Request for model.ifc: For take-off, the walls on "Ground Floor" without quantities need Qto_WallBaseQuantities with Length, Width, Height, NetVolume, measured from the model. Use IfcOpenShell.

First a look at what the model holds.

```python
import ifcopenshell
import ifcopenshell.util.element
import ifcopenshell.util.unit

model = ifcopenshell.open("model.ifc")
print(model.schema)
for unit_type in ("LENGTHUNIT", "AREAUNIT", "VOLUMEUNIT"):
    print(unit_type, ifcopenshell.util.unit.calculate_unit_scale(model, unit_type))
storey = next(s for s in model.by_type("IfcBuildingStorey") if s.Name == "Ground Floor")
walls = [e for e in ifcopenshell.util.element.get_decomposition(storey) if e.is_a("IfcWall")]
for e in sorted(walls, key=lambda e: e.id()):
    print(e.id(), e.is_a(), e.Name, list(ifcopenshell.util.element.get_psets(e, qtos_only=True)), sep=" | ")
```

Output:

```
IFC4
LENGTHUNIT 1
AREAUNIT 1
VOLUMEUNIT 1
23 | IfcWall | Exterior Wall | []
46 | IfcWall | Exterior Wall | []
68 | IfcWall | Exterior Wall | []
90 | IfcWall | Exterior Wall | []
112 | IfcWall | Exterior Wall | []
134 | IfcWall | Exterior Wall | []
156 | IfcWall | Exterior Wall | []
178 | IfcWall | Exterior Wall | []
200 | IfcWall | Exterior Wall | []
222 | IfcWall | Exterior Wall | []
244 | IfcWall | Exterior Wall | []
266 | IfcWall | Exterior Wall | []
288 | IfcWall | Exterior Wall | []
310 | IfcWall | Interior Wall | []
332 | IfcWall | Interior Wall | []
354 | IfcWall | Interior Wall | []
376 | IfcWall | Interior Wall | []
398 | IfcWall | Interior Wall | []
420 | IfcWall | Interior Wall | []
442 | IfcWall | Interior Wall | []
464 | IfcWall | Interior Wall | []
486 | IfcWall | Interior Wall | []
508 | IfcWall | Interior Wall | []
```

```python
import ifcopenshell
import ifcopenshell.api.pset
import ifcopenshell.geom
import ifcopenshell.util.element
import ifcopenshell.util.shape
import ifcopenshell.util.unit

model = ifcopenshell.open("model.ifc")
unit_scale = ifcopenshell.util.unit.calculate_unit_scale(model)
volume_scale = ifcopenshell.util.unit.calculate_unit_scale(model, "VOLUMEUNIT")
settings = ifcopenshell.geom.settings()

storey = next(s for s in model.by_type("IfcBuildingStorey") if s.Name == "Ground Floor")
walls = [e for e in ifcopenshell.util.element.get_decomposition(storey) if e.is_a("IfcWall")]

for e in sorted(walls, key=lambda e: e.id()):
    if ifcopenshell.util.element.get_psets(e, qtos_only=True, should_inherit=False):
        continue
    # Geometry comes back in metres, in the element's own axes.
    shape = ifcopenshell.geom.create_shape(settings, e)
    values = {
        "Length": ifcopenshell.util.shape.get_x(shape.geometry) / unit_scale,
        "Width": ifcopenshell.util.shape.get_y(shape.geometry) / unit_scale,
        "Height": ifcopenshell.util.shape.get_z(shape.geometry) / unit_scale,
        "NetVolume": ifcopenshell.util.shape.get_volume(shape.geometry) / volume_scale,
    }
    qto = ifcopenshell.api.pset.add_qto(model, product=e, name="Qto_WallBaseQuantities")
    ifcopenshell.api.pset.edit_qto(model, qto=qto, properties=values)
    print(e.id(), {k: round(v, 3) for k, v in values.items()})

model.write("model_updated.ifc")
```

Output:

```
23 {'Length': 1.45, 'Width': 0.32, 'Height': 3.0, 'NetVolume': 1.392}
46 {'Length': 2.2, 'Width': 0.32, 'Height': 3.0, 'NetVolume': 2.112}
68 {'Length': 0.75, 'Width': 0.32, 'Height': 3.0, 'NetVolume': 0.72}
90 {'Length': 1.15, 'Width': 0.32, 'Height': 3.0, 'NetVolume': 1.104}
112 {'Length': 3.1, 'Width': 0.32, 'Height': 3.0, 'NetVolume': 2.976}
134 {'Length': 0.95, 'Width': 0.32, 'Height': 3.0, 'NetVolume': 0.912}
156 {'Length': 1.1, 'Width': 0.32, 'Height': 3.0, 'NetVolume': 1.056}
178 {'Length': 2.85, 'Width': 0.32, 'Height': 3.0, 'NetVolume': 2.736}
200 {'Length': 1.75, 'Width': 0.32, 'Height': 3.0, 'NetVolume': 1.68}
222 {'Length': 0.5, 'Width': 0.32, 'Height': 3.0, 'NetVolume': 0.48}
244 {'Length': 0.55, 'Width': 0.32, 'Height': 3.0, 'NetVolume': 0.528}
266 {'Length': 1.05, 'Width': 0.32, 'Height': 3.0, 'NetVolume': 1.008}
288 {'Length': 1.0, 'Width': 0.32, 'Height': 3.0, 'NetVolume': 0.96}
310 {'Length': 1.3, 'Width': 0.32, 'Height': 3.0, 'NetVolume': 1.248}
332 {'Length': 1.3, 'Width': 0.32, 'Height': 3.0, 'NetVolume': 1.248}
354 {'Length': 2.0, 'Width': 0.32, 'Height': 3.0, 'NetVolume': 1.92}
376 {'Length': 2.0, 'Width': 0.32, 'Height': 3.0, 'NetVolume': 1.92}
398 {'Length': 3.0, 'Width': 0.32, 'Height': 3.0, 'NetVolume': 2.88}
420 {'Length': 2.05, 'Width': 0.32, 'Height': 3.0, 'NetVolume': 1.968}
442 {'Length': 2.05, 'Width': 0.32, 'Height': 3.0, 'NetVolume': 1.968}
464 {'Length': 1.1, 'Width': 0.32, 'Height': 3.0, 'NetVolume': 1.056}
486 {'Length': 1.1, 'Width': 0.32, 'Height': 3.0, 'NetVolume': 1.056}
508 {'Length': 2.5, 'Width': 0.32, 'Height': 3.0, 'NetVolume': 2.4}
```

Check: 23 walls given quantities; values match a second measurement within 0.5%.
